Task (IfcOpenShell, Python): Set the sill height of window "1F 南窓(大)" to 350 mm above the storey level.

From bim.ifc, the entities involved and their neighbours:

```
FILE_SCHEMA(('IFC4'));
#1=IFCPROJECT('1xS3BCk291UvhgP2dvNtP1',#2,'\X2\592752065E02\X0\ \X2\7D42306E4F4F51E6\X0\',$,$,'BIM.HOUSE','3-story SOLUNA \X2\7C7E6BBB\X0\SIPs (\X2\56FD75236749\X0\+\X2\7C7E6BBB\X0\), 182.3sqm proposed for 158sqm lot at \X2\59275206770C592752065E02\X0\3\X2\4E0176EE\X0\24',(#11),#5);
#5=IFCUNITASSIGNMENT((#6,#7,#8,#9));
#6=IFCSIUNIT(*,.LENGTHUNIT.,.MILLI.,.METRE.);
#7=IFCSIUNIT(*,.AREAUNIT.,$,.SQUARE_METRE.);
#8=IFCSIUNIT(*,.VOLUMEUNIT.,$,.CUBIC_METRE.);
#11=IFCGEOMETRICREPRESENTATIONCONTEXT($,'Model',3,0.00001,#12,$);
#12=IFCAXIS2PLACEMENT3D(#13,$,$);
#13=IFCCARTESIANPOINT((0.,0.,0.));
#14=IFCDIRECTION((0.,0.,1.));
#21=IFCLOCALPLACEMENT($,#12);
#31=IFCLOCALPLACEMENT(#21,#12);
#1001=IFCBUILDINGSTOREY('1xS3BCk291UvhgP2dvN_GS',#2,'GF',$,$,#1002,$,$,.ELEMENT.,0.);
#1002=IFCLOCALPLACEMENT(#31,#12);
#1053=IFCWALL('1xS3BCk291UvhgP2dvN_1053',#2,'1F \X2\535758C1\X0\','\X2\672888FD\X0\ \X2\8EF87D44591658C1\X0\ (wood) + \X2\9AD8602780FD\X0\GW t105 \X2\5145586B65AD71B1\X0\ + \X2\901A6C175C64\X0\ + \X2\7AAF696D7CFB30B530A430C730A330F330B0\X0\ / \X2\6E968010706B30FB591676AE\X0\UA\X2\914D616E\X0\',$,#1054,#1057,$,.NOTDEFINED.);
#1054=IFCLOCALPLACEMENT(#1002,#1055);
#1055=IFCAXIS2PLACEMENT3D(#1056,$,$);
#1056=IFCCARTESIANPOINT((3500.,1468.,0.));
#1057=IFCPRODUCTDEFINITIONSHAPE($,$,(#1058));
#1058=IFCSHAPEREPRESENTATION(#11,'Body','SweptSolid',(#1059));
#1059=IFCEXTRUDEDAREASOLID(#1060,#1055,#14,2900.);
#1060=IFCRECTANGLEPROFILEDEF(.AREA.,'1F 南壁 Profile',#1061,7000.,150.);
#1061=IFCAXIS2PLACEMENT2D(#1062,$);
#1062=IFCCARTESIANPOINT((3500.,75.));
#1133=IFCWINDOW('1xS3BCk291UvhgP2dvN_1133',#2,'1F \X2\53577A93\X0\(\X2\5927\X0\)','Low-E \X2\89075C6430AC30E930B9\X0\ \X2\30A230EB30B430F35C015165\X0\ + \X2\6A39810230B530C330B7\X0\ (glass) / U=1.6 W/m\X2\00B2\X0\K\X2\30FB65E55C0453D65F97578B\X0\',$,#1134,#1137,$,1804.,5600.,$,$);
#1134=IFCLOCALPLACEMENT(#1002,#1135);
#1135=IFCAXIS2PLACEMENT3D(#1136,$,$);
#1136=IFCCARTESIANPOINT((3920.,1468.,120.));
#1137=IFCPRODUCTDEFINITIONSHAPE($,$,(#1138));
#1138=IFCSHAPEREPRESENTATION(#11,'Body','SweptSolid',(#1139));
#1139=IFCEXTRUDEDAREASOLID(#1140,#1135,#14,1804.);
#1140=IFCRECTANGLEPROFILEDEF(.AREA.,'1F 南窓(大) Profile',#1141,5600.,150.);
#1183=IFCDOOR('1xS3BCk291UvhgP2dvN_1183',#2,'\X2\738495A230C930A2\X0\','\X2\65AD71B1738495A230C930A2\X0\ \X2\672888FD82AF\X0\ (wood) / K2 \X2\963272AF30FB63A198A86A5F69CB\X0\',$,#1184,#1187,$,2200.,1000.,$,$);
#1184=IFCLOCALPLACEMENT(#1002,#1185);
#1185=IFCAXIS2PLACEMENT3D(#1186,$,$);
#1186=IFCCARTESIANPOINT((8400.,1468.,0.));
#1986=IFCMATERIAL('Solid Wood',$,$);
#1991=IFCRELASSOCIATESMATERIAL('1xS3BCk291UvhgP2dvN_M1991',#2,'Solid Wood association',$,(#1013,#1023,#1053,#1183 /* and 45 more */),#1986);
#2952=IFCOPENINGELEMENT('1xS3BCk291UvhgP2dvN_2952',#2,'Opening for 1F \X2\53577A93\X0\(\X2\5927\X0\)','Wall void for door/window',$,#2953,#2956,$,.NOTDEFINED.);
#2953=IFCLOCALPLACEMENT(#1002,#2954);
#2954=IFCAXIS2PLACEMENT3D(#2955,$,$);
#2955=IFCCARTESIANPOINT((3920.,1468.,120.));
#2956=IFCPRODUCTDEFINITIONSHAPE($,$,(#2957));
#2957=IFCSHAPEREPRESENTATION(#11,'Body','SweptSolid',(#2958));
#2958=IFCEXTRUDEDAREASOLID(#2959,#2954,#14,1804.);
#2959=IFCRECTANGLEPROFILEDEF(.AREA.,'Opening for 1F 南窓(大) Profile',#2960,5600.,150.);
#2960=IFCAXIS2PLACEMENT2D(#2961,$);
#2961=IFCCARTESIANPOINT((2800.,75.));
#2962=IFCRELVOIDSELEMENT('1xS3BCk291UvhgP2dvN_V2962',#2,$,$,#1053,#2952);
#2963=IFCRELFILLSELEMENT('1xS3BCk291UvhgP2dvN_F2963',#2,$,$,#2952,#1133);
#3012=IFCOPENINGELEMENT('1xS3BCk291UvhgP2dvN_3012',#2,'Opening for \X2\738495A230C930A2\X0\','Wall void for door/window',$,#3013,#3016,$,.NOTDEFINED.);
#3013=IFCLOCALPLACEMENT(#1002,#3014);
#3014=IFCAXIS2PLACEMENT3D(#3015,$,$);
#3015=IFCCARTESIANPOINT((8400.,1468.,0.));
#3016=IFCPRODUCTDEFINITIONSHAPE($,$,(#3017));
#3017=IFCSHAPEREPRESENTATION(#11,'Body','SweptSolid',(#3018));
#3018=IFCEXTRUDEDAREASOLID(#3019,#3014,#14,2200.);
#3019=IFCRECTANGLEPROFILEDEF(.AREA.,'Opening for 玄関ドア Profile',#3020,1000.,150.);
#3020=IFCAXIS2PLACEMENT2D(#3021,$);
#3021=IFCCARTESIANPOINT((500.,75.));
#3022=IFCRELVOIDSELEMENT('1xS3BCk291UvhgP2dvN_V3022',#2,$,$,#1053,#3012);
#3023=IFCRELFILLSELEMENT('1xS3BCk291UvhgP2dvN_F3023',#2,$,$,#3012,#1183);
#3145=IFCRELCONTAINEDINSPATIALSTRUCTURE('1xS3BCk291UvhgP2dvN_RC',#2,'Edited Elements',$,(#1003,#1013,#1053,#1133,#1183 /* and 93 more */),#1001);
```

```python
import numpy as np
import ifcopenshell
import ifcopenshell.api.geometry
import ifcopenshell.geom
import ifcopenshell.util.element
import ifcopenshell.util.placement
import ifcopenshell.util.shape
import ifcopenshell.util.unit

model = ifcopenshell.open("bim.ifc")
unit_scale = ifcopenshell.util.unit.calculate_unit_scale(model)

window = model.by_id(1133)
opening = window.FillsVoids[0].RelatingOpeningElement
storey = ifcopenshell.util.element.get_container(window, ifc_class="IfcBuildingStorey")
level = ifcopenshell.util.placement.get_local_placement(storey.ObjectPlacement)[2, 3]

# The opening's origin need not be at the sill, so measure its lowest point.
shape = ifcopenshell.geom.create_shape(ifcopenshell.geom.settings(), opening)
bottom = ifcopenshell.util.shape.get_shape_bottom_elevation(shape, shape.geometry) / unit_scale
dz = level + 350.0 - bottom

shift = np.array([0.0, 0.0, dz])
# The window is not placed relative to its opening, so move both.
for product in (opening, window):
    matrix = ifcopenshell.util.placement.get_local_placement(product.ObjectPlacement)
    matrix[:3, 3] += shift
    ifcopenshell.api.geometry.edit_object_placement(model, product=product, matrix=matrix, is_si=False)

print(f"moved by {dz * unit_scale:+.3f} m")

model.write("bim_edited.ifc")
```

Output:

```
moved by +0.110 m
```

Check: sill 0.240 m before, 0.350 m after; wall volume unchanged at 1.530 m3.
